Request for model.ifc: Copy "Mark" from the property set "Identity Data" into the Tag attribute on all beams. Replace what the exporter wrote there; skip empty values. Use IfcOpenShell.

First a look at what the model holds.

```python
import ifcopenshell
import ifcopenshell.util.element

model = ifcopenshell.open("model.ifc")
print(model.schema)
beams = model.by_type("IfcBeam")
print(len(beams), "beams")
for e in beams[:8]:
    source = ifcopenshell.util.element.get_pset(e, "Identity Data", "Mark")
    target = e.Tag
    print(e.id(), repr(source), repr(target), sep=" | ")
```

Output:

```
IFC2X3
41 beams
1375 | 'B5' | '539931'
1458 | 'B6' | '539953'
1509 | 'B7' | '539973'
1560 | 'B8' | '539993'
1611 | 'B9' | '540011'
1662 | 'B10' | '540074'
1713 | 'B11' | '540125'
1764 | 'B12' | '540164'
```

```python
import ifcopenshell
import ifcopenshell.util.element

model = ifcopenshell.open("model.ifc")

count = 0
for e in model.by_type("IfcBeam"):
    value = ifcopenshell.util.element.get_pset(e, "Identity Data", "Mark")
    current = e.Tag
    if not value or not value.strip() or current == value:
        continue
    e.Tag = value
    count += 1

print(count, "beams updated")

model.write("model-out.ifc")
```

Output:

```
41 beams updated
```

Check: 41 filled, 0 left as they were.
